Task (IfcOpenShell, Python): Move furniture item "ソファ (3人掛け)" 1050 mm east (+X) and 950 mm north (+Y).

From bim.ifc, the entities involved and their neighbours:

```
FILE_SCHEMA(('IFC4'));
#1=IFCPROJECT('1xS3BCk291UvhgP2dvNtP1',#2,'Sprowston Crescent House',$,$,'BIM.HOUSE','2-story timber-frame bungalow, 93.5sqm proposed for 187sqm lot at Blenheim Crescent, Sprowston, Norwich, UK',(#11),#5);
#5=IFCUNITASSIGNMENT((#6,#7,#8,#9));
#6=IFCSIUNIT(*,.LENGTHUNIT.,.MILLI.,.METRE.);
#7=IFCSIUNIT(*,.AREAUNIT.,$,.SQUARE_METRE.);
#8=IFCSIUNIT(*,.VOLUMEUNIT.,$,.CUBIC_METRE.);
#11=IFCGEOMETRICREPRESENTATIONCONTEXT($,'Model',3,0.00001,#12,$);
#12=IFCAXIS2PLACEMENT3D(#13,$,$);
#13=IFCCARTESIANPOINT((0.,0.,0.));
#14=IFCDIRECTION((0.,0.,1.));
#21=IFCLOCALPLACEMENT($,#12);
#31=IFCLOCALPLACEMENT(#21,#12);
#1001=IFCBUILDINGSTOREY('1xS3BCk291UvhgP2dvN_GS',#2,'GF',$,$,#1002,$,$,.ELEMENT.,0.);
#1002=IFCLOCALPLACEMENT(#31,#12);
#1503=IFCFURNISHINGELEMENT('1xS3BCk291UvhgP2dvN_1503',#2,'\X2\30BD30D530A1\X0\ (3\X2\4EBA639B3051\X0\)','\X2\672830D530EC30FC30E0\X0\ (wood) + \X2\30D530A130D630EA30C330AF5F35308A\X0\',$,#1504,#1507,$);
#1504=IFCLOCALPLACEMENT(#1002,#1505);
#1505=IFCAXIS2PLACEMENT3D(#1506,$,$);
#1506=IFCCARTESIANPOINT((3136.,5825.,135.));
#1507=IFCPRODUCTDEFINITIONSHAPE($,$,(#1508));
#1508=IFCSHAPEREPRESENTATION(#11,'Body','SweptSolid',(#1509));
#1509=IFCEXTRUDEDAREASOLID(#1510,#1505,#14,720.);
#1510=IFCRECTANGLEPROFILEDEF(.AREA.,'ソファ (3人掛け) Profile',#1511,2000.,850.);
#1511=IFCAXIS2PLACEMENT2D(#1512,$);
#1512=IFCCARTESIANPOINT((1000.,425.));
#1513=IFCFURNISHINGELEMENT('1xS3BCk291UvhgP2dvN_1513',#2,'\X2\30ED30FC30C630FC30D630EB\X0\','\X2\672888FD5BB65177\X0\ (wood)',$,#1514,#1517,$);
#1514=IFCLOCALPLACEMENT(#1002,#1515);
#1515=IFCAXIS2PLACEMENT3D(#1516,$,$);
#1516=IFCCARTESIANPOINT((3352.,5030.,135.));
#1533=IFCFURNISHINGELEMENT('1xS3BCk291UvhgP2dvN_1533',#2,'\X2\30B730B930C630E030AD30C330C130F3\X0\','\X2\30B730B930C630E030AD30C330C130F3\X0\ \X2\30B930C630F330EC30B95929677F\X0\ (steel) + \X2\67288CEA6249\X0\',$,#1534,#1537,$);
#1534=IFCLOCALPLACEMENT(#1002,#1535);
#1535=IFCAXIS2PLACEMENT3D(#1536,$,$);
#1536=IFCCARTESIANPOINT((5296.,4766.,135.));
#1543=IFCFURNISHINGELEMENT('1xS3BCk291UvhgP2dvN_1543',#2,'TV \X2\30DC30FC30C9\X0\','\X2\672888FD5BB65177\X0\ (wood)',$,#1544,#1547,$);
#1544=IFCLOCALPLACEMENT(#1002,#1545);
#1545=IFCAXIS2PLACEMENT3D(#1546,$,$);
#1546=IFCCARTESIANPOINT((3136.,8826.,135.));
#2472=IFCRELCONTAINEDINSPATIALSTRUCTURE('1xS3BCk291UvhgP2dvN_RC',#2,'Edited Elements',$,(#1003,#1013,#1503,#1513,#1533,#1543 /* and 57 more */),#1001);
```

```python
import ifcopenshell
import ifcopenshell.api.geometry
import ifcopenshell.util.placement

model = ifcopenshell.open("bim.ifc")

item = model.by_id(1503)
matrix = ifcopenshell.util.placement.get_local_placement(item.ObjectPlacement)
matrix[0, 3] += 1050.0
matrix[1, 3] += 950.0
ifcopenshell.api.geometry.edit_object_placement(model, product=item, matrix=matrix, is_si=False)

print(ifcopenshell.util.placement.get_local_placement(item.ObjectPlacement).round(3) + 0.0)

model.write("bim_v2.ifc")
```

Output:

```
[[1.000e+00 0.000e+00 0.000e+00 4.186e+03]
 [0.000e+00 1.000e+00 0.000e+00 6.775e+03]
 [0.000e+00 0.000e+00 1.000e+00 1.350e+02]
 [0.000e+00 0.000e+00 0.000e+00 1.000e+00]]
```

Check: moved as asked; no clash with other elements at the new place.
